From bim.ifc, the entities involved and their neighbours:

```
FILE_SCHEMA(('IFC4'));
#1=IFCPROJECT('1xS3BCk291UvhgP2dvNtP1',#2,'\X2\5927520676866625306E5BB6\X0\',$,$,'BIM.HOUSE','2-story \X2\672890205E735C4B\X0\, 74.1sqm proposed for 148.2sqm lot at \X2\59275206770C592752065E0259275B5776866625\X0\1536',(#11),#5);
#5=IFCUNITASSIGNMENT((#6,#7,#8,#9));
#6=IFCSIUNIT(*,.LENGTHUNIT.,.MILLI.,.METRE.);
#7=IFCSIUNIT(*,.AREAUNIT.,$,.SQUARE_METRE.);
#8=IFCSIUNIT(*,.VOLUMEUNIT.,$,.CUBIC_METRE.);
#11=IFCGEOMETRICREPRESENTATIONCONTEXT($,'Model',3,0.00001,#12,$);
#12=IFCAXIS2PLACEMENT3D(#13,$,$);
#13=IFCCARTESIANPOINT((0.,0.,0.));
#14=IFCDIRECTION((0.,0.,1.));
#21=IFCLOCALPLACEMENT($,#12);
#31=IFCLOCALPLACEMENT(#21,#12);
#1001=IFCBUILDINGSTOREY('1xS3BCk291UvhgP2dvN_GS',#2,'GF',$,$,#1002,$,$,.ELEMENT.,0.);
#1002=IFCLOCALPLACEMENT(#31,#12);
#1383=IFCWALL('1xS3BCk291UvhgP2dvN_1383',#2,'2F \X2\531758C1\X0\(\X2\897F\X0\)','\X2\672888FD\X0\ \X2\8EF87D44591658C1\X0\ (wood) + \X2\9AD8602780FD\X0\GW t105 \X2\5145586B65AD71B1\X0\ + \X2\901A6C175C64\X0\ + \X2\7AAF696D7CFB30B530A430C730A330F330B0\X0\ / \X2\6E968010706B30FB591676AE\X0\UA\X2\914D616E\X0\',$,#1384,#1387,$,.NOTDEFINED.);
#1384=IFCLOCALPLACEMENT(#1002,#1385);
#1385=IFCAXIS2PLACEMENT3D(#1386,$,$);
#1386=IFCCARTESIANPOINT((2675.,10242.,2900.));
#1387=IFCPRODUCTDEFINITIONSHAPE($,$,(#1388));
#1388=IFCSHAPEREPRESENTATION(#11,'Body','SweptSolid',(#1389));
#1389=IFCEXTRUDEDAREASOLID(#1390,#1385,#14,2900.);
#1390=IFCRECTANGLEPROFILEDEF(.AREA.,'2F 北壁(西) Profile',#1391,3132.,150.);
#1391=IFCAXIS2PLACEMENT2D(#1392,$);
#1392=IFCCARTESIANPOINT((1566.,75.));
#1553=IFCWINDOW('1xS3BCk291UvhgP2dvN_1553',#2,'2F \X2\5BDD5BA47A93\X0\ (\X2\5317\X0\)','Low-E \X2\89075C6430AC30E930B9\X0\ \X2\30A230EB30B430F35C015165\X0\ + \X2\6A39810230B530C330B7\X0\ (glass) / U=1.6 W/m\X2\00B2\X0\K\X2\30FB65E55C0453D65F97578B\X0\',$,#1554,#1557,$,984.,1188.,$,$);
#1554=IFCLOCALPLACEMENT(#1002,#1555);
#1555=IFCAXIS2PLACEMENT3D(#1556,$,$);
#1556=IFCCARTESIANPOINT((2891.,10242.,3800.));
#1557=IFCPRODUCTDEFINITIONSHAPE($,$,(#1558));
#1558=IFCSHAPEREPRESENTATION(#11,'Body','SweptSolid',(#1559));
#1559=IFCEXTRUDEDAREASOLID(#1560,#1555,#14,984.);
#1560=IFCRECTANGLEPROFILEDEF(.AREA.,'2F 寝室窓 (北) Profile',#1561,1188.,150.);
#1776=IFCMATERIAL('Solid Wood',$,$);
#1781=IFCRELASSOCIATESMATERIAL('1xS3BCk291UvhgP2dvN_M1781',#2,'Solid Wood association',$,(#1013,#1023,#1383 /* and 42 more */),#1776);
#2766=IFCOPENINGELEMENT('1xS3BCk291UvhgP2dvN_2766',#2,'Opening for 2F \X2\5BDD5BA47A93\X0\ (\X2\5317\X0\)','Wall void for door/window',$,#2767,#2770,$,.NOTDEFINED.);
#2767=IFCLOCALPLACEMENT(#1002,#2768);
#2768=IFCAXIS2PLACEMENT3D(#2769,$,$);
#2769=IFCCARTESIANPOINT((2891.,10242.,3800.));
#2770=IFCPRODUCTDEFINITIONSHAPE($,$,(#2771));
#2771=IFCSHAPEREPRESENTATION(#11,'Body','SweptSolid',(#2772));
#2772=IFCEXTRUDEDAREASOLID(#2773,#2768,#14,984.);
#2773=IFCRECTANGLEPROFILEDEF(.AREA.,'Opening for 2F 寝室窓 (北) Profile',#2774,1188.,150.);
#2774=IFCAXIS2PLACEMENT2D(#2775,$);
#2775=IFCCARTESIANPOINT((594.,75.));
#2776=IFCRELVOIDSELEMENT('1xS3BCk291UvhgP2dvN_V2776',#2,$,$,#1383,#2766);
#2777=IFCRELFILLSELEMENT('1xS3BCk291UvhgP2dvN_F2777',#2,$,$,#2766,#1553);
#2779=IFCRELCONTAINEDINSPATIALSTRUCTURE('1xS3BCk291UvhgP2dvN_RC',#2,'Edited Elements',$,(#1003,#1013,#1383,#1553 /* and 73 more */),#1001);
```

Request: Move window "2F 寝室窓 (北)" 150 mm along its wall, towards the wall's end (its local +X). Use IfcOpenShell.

```python
import ifcopenshell
import ifcopenshell.api.geometry
import ifcopenshell.util.placement
import ifcopenshell.util.unit

model = ifcopenshell.open("bim.ifc")
unit_scale = ifcopenshell.util.unit.calculate_unit_scale(model)

window = model.by_guid("1xS3BCk291UvhgP2dvN_1553")
opening = window.FillsVoids[0].RelatingOpeningElement
wall = opening.VoidsElements[0].RelatingBuildingElement

wall_matrix = ifcopenshell.util.placement.get_local_placement(wall.ObjectPlacement)
shift = wall_matrix[:3, 0] * 0.15 / unit_scale
before = ifcopenshell.util.placement.get_local_placement(window.ObjectPlacement)[:3, 3].copy()

# The window is not placed relative to its opening, so move both.
for product in (opening, window):
    matrix = ifcopenshell.util.placement.get_local_placement(product.ObjectPlacement)
    matrix[:3, 3] += shift
    ifcopenshell.api.geometry.edit_object_placement(model, product=product, matrix=matrix, is_si=False)

after = ifcopenshell.util.placement.get_local_placement(window.ObjectPlacement)[:3, 3]
print("window moved by", (after - before).round(3) + 0.0)

model.write("bim-out.ifc")
```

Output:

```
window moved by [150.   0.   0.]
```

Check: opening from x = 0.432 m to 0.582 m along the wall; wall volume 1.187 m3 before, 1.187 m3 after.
